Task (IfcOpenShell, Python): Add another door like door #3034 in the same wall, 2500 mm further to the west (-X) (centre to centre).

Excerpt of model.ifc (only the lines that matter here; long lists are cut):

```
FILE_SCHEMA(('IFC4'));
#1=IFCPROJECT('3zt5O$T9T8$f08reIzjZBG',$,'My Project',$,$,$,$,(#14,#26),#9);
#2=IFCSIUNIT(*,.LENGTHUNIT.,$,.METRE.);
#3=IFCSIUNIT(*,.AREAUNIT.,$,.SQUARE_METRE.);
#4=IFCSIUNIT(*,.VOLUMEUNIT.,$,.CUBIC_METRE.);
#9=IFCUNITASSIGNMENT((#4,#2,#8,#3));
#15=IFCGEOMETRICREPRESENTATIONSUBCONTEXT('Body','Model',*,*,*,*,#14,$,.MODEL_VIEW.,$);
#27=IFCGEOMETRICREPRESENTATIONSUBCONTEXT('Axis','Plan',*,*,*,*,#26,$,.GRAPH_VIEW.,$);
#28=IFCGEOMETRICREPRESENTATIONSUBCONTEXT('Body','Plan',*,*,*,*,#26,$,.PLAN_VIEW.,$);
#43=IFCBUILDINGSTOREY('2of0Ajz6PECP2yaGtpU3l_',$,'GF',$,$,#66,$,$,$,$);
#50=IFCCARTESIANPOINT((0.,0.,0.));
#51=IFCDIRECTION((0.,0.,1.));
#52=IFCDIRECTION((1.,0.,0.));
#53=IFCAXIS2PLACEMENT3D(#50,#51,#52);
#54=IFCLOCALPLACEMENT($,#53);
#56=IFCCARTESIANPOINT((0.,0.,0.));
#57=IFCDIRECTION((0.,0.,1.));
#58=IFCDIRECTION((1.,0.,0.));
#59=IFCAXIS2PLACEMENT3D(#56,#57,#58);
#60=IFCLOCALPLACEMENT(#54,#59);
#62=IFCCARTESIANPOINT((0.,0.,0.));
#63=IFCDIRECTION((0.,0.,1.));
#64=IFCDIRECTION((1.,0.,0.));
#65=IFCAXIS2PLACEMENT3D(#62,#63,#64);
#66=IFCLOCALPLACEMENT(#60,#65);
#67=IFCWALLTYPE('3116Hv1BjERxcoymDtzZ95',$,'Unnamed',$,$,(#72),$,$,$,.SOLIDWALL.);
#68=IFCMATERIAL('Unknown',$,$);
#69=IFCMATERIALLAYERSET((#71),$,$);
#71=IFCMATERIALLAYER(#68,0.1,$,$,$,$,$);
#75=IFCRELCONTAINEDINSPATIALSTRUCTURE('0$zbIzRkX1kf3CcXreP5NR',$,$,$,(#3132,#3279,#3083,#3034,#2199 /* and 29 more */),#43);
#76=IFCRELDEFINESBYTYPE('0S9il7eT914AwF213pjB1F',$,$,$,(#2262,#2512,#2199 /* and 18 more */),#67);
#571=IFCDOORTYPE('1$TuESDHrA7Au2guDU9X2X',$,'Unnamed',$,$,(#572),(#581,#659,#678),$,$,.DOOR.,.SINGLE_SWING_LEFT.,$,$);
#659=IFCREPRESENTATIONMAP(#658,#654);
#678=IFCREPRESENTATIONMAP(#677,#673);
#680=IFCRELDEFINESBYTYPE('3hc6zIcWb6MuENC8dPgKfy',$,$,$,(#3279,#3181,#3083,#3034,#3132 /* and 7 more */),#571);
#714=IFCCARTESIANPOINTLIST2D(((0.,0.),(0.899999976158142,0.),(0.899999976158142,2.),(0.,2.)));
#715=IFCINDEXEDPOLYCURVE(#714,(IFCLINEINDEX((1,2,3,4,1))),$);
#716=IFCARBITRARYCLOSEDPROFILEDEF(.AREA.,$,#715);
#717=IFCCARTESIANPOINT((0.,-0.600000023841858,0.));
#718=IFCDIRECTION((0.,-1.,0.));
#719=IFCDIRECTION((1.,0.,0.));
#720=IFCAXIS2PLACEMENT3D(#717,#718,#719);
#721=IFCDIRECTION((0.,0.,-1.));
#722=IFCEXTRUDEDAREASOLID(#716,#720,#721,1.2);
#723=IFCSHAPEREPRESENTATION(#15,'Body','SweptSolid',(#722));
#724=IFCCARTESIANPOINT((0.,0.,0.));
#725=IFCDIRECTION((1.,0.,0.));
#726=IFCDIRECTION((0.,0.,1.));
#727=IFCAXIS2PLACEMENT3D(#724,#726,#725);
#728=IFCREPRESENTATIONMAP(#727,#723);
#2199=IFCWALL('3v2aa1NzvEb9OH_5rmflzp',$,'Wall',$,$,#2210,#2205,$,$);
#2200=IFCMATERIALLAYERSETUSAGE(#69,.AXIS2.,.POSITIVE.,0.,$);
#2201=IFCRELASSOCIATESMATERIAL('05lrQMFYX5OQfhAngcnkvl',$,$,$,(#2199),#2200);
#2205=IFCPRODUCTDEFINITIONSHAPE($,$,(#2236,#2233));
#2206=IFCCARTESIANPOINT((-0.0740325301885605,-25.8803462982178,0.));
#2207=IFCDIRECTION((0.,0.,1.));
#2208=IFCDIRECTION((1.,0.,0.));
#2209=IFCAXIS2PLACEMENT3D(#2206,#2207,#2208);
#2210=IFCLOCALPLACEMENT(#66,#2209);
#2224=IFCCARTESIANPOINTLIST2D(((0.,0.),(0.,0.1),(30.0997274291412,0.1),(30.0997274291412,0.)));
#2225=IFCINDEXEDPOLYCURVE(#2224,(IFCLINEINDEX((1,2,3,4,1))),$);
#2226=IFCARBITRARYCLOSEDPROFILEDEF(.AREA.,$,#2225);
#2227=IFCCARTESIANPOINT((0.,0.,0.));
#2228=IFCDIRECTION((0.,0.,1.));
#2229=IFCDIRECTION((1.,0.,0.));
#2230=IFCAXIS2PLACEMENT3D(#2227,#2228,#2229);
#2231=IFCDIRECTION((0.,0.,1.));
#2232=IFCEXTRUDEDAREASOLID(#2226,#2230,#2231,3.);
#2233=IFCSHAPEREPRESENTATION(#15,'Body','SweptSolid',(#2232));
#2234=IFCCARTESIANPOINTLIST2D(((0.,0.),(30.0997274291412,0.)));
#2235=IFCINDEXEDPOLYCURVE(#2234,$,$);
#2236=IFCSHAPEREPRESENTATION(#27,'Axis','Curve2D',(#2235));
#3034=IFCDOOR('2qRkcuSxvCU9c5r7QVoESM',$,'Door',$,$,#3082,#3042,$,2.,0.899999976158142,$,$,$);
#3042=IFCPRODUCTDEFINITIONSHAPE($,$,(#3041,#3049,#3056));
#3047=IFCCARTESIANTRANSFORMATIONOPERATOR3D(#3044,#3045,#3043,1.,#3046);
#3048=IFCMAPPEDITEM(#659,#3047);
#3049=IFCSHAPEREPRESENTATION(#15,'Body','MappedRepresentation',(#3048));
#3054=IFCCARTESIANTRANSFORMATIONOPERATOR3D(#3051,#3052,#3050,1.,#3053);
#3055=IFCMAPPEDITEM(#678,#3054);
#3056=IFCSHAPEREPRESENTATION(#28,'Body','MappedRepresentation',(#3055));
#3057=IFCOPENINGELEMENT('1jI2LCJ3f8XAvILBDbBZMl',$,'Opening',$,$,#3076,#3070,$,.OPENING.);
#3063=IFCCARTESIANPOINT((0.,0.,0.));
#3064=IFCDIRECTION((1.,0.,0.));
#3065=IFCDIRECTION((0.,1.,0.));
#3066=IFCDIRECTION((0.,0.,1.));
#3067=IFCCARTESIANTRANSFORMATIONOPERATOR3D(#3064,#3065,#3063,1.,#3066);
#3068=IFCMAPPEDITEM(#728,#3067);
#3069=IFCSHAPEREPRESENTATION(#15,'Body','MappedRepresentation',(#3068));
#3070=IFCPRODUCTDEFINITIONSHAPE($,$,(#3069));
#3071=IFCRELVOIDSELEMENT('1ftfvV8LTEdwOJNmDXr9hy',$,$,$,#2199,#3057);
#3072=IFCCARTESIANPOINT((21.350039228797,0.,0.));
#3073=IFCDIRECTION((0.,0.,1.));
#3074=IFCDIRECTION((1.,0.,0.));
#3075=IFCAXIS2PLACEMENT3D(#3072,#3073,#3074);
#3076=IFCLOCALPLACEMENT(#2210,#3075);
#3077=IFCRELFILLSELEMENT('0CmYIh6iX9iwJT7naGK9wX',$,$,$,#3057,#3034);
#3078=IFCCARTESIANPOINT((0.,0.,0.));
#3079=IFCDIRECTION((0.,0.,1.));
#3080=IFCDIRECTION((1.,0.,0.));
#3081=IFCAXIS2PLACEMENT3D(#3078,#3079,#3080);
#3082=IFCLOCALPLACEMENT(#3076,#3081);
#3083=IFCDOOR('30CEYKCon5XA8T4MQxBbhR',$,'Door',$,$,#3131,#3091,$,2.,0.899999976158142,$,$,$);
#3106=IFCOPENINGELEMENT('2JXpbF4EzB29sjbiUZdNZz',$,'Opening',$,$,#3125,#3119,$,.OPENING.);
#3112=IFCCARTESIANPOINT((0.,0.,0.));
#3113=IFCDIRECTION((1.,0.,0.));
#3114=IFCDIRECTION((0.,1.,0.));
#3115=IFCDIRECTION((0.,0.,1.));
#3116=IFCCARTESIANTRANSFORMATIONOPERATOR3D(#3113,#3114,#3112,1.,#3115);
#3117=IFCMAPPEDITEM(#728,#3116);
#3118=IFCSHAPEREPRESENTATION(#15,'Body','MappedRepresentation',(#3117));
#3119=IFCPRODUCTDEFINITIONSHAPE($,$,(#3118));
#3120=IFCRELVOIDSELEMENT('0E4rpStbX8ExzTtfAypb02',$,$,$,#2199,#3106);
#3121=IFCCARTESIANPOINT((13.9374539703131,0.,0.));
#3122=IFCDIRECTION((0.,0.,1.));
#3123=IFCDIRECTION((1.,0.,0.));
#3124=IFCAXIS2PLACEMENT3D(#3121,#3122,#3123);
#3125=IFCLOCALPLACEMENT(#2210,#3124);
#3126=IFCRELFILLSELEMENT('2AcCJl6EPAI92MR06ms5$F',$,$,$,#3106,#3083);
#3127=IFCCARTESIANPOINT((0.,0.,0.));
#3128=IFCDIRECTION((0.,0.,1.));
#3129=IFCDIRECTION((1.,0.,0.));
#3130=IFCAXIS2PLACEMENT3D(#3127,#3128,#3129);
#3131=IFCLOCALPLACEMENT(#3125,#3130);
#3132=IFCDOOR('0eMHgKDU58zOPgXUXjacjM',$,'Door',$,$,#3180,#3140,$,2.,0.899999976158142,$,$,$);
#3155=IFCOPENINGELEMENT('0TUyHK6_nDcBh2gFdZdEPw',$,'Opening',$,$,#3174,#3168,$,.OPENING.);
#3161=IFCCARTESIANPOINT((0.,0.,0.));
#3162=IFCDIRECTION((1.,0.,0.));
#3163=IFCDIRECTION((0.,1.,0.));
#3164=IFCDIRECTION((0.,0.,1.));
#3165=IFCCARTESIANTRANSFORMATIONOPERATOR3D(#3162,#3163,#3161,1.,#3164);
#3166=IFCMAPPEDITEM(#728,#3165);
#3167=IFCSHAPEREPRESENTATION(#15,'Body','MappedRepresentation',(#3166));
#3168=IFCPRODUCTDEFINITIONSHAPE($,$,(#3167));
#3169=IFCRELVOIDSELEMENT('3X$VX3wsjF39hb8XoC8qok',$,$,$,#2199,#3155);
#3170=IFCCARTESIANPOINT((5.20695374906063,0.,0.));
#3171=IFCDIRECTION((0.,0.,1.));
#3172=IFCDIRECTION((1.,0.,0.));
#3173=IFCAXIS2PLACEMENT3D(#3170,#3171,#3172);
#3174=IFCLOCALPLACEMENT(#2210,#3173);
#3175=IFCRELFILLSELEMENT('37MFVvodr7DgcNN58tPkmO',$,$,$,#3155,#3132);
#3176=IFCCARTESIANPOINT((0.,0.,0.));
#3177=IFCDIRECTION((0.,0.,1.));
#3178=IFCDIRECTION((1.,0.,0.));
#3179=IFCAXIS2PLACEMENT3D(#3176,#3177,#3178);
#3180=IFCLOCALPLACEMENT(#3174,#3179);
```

```python
import ifcopenshell
import ifcopenshell.api.feature
import ifcopenshell.api.geometry
import ifcopenshell.api.root
import ifcopenshell.geom
import ifcopenshell.util.element
import ifcopenshell.util.placement
import ifcopenshell.util.shape

model = ifcopenshell.open("model.ifc")
settings = ifcopenshell.geom.settings()


def volume(element):
    """Net volume in cubic metres, openings subtracted."""
    shape = ifcopenshell.geom.create_shape(settings, element)
    return ifcopenshell.util.shape.get_volume(shape.geometry)


door = model.by_id(3034)
opening = door.FillsVoids[0].RelatingOpeningElement
wall = opening.VoidsElements[0].RelatingBuildingElement
before = volume(wall)
shift = ifcopenshell.util.placement.get_local_placement(wall.ObjectPlacement)[:3, 0] * -2.5

# copy_class copies the void relationship, type, container and properties, but no geometry.
new_opening = ifcopenshell.api.root.copy_class(model, product=opening)
new_opening.Representation = ifcopenshell.util.element.copy_deep(
    model, opening.Representation, exclude=["IfcGeometricRepresentationContext", "IfcRepresentationMap"]
)
new_door = ifcopenshell.api.root.copy_class(model, product=door)
new_door.Representation = ifcopenshell.util.element.copy_deep(
    model, door.Representation, exclude=["IfcGeometricRepresentationContext", "IfcRepresentationMap"]
)
ifcopenshell.api.feature.add_filling(model, opening=new_opening, element=new_door)

for old, new in ((opening, new_opening), (door, new_door)):
    matrix = ifcopenshell.util.placement.get_local_placement(old.ObjectPlacement)
    matrix[:3, 3] += shift
    ifcopenshell.api.geometry.edit_object_placement(model, product=new, matrix=matrix, is_si=False)

after = volume(wall)

print(f"wall volume {before:.3f} -> {after:.3f} m3")

model.write("model_v2.ifc")
```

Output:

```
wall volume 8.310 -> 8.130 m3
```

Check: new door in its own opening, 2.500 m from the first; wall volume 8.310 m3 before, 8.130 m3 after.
